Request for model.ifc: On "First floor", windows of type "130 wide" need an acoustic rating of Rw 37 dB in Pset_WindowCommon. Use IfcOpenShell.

First a look at what the model holds.

```python
import ifcopenshell
import ifcopenshell.util.element

model = ifcopenshell.open("model.ifc")
print(model.schema)
storey = next(s for s in model.by_type("IfcBuildingStorey") if s.Name == "First floor")
windows = [e for e in ifcopenshell.util.element.get_decomposition(storey) if e.is_a("IfcWindow")]
seen = {}
for e in windows:
    element_type = ifcopenshell.util.element.get_type(e)
    key = (element_type.Name if element_type != e and element_type else None, ifcopenshell.util.element.get_pset(e, "Pset_WindowCommon", "AcousticRating"))
    seen[key] = seen.get(key, 0) + 1
for (name, value), count in sorted(seen.items(), key=str):
    print(count, "x", name, "|", value)
```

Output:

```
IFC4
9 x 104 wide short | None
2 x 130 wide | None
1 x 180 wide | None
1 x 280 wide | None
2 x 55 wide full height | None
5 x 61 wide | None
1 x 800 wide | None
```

```python
import ifcopenshell
import ifcopenshell.api.pset
import ifcopenshell.util.element

model = ifcopenshell.open("model.ifc")

storey = next(s for s in model.by_type("IfcBuildingStorey") if s.Name == "First floor")
windows = [e for e in ifcopenshell.util.element.get_decomposition(storey) if e.is_a("IfcWindow")]

count = 0
for e in windows:
    element_type = ifcopenshell.util.element.get_type(e)
    if element_type in (None, e) or element_type.Name != "130 wide":
        continue
    # add_pset returns the element's existing set when there is one.
    pset = ifcopenshell.api.pset.add_pset(model, product=e, name="Pset_WindowCommon")
    ifcopenshell.api.pset.edit_pset(model, pset=pset, properties={"AcousticRating": "Rw 37 dB"})
    count += 1

print(count, "windows updated")

model.write("model_updated.ifc")
```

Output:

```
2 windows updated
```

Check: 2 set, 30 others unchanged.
